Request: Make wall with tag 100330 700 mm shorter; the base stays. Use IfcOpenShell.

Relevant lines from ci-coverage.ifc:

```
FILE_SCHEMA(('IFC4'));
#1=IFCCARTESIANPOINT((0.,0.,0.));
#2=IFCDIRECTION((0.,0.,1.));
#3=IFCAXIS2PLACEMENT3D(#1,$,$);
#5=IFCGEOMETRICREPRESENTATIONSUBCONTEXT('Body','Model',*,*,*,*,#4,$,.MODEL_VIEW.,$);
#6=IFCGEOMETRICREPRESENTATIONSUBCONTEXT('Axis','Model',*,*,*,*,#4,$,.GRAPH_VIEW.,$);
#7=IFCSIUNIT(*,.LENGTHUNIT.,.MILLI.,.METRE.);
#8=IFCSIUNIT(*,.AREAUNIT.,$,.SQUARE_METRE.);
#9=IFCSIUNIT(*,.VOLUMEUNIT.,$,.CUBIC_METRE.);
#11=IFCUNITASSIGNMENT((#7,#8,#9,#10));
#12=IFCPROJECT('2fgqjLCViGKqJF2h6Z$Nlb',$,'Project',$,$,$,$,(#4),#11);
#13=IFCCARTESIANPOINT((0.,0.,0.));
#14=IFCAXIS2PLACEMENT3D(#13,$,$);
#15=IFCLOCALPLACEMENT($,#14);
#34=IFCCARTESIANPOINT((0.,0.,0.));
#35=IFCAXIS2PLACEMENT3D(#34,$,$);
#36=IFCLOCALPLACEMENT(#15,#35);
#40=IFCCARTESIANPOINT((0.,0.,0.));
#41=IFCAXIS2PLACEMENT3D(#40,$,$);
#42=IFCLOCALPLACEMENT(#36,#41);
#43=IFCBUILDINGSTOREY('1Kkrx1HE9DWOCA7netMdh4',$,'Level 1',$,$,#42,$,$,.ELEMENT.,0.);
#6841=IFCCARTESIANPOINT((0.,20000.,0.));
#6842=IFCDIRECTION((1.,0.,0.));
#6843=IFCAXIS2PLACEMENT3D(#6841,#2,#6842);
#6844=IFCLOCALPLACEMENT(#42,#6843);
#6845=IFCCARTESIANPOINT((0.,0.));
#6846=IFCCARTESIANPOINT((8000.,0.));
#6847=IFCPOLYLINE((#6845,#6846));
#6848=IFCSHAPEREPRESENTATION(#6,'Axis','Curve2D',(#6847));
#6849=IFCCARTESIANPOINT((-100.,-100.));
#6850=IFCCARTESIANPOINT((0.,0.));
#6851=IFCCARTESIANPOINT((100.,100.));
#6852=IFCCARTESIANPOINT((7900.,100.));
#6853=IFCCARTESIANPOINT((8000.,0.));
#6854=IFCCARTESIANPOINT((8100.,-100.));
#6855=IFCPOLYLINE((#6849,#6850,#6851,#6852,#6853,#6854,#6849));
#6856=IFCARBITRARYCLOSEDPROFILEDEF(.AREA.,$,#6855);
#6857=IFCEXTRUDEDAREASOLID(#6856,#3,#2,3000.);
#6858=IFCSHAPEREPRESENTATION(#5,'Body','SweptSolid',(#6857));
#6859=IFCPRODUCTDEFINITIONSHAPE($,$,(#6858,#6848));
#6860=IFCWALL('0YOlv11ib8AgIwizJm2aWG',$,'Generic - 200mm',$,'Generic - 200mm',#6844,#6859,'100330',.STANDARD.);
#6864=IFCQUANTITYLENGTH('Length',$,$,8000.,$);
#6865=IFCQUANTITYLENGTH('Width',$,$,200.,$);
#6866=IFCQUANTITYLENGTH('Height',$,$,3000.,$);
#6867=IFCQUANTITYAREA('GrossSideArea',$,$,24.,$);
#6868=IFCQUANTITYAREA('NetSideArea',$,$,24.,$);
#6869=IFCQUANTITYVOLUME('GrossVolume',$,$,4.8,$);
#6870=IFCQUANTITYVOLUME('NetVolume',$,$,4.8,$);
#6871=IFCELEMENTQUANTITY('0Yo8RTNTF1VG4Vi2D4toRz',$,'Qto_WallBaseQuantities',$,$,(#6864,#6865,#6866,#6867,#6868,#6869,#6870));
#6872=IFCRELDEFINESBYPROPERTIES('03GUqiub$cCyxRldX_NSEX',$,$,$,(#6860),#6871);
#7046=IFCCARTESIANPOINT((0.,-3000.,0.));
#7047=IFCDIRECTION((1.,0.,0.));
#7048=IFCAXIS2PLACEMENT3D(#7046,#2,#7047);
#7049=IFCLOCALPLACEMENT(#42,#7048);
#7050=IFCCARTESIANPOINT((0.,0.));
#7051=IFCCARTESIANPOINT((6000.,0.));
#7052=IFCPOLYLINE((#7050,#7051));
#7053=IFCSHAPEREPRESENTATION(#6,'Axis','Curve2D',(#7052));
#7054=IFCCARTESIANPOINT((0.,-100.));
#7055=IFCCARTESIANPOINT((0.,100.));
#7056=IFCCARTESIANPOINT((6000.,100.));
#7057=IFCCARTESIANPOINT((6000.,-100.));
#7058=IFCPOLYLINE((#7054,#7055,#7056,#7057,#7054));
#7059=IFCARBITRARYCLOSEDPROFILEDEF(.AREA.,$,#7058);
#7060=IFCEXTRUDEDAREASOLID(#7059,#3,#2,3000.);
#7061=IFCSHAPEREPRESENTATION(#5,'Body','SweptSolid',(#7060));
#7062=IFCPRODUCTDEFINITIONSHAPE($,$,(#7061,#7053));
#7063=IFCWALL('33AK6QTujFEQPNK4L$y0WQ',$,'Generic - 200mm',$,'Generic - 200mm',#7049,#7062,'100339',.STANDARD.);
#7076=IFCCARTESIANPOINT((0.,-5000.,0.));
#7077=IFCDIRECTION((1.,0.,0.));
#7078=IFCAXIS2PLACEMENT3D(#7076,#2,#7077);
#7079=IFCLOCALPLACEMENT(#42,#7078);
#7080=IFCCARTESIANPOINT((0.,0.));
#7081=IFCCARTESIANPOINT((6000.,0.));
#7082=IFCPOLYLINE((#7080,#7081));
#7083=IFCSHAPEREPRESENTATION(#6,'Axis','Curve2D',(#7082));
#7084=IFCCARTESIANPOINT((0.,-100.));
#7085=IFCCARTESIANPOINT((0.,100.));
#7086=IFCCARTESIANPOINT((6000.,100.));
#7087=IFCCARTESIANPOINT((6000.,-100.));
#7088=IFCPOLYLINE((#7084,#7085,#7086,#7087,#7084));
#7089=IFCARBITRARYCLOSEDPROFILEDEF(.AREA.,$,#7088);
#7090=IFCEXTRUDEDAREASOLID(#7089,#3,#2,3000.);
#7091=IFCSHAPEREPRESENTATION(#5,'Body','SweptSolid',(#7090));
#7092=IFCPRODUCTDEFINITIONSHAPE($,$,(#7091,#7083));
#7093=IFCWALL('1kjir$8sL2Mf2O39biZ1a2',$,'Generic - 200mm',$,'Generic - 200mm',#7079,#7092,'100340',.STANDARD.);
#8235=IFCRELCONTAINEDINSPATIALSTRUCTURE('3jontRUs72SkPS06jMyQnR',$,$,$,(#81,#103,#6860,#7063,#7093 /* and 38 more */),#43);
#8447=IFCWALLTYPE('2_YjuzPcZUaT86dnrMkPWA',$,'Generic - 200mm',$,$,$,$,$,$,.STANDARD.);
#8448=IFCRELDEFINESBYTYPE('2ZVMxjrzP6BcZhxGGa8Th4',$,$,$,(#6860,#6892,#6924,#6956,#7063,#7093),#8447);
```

```python
import ifcopenshell
import ifcopenshell.api.pset
import ifcopenshell.geom
import ifcopenshell.util.element
import ifcopenshell.util.representation
import ifcopenshell.util.shape
import ifcopenshell.util.unit

model = ifcopenshell.open("ci-coverage.ifc")
unit_scale = ifcopenshell.util.unit.calculate_unit_scale(model)
area_scale = ifcopenshell.util.unit.calculate_unit_scale(model, "AREAUNIT")
volume_scale = ifcopenshell.util.unit.calculate_unit_scale(model, "VOLUMEUNIT")
settings = ifcopenshell.geom.settings()


def volume(element):
    """Net volume in cubic metres, openings subtracted."""
    shape = ifcopenshell.geom.create_shape(settings, element)
    return ifcopenshell.util.shape.get_volume(shape.geometry)


wall = model.by_guid("0YOlv11ib8AgIwizJm2aWG")
before = volume(wall)

body = ifcopenshell.util.representation.get_representation(wall, "Model", "Body")
solid = body.Items[0]
old_height = solid.Depth
solid.Depth -= 0.7 / unit_scale
after = volume(wall)
thickness = 0.2  # wall thickness in metres

# Update the stored height, areas and volumes.
qto = model.by_id(ifcopenshell.util.element.get_pset(wall, "Qto_WallBaseQuantities", should_inherit=False)["id"])
ifcopenshell.api.pset.edit_qto(model, qto=qto, properties={
    "Height": solid.Depth,
    "GrossSideArea": ifcopenshell.util.element.get_pset(wall, "Qto_WallBaseQuantities", "GrossSideArea") * solid.Depth / old_height,
    "NetSideArea": after / thickness / area_scale,
    "GrossVolume": ifcopenshell.util.element.get_pset(wall, "Qto_WallBaseQuantities", "GrossVolume") * solid.Depth / old_height,
    "NetVolume": after / volume_scale,
})

print(f"height {old_height:g} -> {solid.Depth:g}, volume {before:.3f} -> {after:.3f} m3")

model.write("ci-coverage_v2.ifc")
```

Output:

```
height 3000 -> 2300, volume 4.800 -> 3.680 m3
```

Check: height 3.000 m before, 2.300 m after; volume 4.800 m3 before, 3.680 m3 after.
